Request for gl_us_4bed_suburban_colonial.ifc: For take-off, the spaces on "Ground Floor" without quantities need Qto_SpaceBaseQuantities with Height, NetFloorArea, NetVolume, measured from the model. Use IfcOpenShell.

First a look at what the model holds.

```python
import ifcopenshell
import ifcopenshell.util.element
import ifcopenshell.util.unit

model = ifcopenshell.open("gl_us_4bed_suburban_colonial.ifc")
print(model.schema)
for unit_type in ("LENGTHUNIT", "AREAUNIT", "VOLUMEUNIT"):
    print(unit_type, ifcopenshell.util.unit.calculate_unit_scale(model, unit_type))
storey = next(s for s in model.by_type("IfcBuildingStorey") if s.Name == "Ground Floor")
spaces = [e for e in ifcopenshell.util.element.get_decomposition(storey) if e.is_a("IfcSpace")]
for e in sorted(spaces, key=lambda e: e.id()):
    print(e.id(), e.is_a(), e.Name, list(ifcopenshell.util.element.get_psets(e, qtos_only=True)), sep=" | ")
```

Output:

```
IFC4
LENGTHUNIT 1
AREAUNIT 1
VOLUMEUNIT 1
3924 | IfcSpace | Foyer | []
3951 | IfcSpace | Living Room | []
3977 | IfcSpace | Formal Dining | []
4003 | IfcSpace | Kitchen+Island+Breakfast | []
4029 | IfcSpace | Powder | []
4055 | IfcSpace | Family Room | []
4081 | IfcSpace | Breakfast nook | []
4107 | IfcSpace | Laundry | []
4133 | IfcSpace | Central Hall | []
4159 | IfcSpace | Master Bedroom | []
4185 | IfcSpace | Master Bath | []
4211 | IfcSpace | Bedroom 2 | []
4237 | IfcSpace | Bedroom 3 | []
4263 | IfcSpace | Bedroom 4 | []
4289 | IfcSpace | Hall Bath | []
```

```python
import ifcopenshell
import ifcopenshell.api.pset
import ifcopenshell.geom
import ifcopenshell.util.element
import ifcopenshell.util.shape
import ifcopenshell.util.unit

model = ifcopenshell.open("gl_us_4bed_suburban_colonial.ifc")
unit_scale = ifcopenshell.util.unit.calculate_unit_scale(model)
area_scale = ifcopenshell.util.unit.calculate_unit_scale(model, "AREAUNIT")
volume_scale = ifcopenshell.util.unit.calculate_unit_scale(model, "VOLUMEUNIT")
settings = ifcopenshell.geom.settings()

storey = next(s for s in model.by_type("IfcBuildingStorey") if s.Name == "Ground Floor")
spaces = [e for e in ifcopenshell.util.element.get_decomposition(storey) if e.is_a("IfcSpace")]

for e in sorted(spaces, key=lambda e: e.id()):
    if ifcopenshell.util.element.get_psets(e, qtos_only=True, should_inherit=False):
        continue
    # Geometry comes back in metres, in the element's own axes.
    shape = ifcopenshell.geom.create_shape(settings, e)
    values = {
        "Height": ifcopenshell.util.shape.get_z(shape.geometry) / unit_scale,
        "NetFloorArea": ifcopenshell.util.shape.get_footprint_area(shape.geometry) / area_scale,
        "NetVolume": ifcopenshell.util.shape.get_volume(shape.geometry) / volume_scale,
    }
    qto = ifcopenshell.api.pset.add_qto(model, product=e, name="Qto_SpaceBaseQuantities")
    ifcopenshell.api.pset.edit_qto(model, qto=qto, properties=values)
    print(e.id(), {k: round(v, 3) for k, v in values.items()})

model.write("gl_us_4bed_suburban_colonial_updated.ifc")
```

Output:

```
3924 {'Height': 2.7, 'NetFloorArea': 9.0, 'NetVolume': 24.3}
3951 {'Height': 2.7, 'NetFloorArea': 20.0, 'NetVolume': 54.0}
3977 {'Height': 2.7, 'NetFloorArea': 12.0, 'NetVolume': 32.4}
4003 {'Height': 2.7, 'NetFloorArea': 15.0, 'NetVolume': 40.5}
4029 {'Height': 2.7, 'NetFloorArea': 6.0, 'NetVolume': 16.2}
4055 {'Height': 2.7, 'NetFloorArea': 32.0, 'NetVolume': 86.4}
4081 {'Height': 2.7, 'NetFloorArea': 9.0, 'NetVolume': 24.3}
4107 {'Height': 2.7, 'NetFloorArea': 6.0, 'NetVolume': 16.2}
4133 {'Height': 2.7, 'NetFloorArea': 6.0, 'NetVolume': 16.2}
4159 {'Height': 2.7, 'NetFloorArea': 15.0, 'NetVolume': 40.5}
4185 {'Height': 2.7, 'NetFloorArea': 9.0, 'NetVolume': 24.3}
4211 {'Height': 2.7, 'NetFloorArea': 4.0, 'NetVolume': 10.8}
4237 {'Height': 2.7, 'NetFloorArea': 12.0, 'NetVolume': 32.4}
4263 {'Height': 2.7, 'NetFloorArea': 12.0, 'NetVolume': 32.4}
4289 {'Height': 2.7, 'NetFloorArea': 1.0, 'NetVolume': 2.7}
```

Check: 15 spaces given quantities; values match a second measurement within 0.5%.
